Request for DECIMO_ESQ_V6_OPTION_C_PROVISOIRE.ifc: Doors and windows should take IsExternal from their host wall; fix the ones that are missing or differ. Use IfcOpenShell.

First a look at what the model holds.

```python
import ifcopenshell
import ifcopenshell.util.element

model = ifcopenshell.open("DECIMO_ESQ_V6_OPTION_C_PROVISOIRE.ifc")
print(model.schema)
seen = {}
for e in model.by_type("IfcDoor") + model.by_type("IfcWindow"):
    if not e.FillsVoids:
        continue
    host = e.FillsVoids[0].RelatingOpeningElement.VoidsElements[0].RelatingBuildingElement
    own = ifcopenshell.util.element.get_pset(e, f"Pset_{e.is_a()[3:].removesuffix('StandardCase')}Common", "IsExternal")
    wall = ifcopenshell.util.element.get_pset(host, "Pset_WallCommon", "IsExternal")
    seen[e.is_a(), own, wall] = seen.get((e.is_a(), own, wall), 0) + 1
for (cls, own, wall), count in sorted(seen.items(), key=str):
    print(count, cls, "IsExternal:", own, "| host wall:", wall)
```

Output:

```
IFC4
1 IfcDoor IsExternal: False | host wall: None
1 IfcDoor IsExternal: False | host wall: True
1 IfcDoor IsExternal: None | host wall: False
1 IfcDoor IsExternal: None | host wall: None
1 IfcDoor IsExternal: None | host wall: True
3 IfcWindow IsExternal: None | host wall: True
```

```python
import ifcopenshell
import ifcopenshell.api.pset
import ifcopenshell.util.element

model = ifcopenshell.open("DECIMO_ESQ_V6_OPTION_C_PROVISOIRE.ifc")

count = 0
for ifc_class, pset_name in (("IfcDoor", "Pset_DoorCommon"), ("IfcWindow", "Pset_WindowCommon")):
    for e in model.by_type(ifc_class):
        if not e.FillsVoids:
            continue
        host = e.FillsVoids[0].RelatingOpeningElement.VoidsElements[0].RelatingBuildingElement
        external = ifcopenshell.util.element.get_pset(host, "Pset_WallCommon", "IsExternal")
        if external is None or ifcopenshell.util.element.get_pset(e, pset_name, "IsExternal") == external:
            continue
        pset = ifcopenshell.api.pset.add_pset(model, product=e, name=pset_name)
        ifcopenshell.api.pset.edit_pset(model, pset=pset, properties={"IsExternal": external})
        count += 1

print(count, "updated")

model.write("DECIMO_ESQ_V6_OPTION_C_PROVISOIRE_rev.ifc")
```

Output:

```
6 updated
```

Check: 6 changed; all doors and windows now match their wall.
